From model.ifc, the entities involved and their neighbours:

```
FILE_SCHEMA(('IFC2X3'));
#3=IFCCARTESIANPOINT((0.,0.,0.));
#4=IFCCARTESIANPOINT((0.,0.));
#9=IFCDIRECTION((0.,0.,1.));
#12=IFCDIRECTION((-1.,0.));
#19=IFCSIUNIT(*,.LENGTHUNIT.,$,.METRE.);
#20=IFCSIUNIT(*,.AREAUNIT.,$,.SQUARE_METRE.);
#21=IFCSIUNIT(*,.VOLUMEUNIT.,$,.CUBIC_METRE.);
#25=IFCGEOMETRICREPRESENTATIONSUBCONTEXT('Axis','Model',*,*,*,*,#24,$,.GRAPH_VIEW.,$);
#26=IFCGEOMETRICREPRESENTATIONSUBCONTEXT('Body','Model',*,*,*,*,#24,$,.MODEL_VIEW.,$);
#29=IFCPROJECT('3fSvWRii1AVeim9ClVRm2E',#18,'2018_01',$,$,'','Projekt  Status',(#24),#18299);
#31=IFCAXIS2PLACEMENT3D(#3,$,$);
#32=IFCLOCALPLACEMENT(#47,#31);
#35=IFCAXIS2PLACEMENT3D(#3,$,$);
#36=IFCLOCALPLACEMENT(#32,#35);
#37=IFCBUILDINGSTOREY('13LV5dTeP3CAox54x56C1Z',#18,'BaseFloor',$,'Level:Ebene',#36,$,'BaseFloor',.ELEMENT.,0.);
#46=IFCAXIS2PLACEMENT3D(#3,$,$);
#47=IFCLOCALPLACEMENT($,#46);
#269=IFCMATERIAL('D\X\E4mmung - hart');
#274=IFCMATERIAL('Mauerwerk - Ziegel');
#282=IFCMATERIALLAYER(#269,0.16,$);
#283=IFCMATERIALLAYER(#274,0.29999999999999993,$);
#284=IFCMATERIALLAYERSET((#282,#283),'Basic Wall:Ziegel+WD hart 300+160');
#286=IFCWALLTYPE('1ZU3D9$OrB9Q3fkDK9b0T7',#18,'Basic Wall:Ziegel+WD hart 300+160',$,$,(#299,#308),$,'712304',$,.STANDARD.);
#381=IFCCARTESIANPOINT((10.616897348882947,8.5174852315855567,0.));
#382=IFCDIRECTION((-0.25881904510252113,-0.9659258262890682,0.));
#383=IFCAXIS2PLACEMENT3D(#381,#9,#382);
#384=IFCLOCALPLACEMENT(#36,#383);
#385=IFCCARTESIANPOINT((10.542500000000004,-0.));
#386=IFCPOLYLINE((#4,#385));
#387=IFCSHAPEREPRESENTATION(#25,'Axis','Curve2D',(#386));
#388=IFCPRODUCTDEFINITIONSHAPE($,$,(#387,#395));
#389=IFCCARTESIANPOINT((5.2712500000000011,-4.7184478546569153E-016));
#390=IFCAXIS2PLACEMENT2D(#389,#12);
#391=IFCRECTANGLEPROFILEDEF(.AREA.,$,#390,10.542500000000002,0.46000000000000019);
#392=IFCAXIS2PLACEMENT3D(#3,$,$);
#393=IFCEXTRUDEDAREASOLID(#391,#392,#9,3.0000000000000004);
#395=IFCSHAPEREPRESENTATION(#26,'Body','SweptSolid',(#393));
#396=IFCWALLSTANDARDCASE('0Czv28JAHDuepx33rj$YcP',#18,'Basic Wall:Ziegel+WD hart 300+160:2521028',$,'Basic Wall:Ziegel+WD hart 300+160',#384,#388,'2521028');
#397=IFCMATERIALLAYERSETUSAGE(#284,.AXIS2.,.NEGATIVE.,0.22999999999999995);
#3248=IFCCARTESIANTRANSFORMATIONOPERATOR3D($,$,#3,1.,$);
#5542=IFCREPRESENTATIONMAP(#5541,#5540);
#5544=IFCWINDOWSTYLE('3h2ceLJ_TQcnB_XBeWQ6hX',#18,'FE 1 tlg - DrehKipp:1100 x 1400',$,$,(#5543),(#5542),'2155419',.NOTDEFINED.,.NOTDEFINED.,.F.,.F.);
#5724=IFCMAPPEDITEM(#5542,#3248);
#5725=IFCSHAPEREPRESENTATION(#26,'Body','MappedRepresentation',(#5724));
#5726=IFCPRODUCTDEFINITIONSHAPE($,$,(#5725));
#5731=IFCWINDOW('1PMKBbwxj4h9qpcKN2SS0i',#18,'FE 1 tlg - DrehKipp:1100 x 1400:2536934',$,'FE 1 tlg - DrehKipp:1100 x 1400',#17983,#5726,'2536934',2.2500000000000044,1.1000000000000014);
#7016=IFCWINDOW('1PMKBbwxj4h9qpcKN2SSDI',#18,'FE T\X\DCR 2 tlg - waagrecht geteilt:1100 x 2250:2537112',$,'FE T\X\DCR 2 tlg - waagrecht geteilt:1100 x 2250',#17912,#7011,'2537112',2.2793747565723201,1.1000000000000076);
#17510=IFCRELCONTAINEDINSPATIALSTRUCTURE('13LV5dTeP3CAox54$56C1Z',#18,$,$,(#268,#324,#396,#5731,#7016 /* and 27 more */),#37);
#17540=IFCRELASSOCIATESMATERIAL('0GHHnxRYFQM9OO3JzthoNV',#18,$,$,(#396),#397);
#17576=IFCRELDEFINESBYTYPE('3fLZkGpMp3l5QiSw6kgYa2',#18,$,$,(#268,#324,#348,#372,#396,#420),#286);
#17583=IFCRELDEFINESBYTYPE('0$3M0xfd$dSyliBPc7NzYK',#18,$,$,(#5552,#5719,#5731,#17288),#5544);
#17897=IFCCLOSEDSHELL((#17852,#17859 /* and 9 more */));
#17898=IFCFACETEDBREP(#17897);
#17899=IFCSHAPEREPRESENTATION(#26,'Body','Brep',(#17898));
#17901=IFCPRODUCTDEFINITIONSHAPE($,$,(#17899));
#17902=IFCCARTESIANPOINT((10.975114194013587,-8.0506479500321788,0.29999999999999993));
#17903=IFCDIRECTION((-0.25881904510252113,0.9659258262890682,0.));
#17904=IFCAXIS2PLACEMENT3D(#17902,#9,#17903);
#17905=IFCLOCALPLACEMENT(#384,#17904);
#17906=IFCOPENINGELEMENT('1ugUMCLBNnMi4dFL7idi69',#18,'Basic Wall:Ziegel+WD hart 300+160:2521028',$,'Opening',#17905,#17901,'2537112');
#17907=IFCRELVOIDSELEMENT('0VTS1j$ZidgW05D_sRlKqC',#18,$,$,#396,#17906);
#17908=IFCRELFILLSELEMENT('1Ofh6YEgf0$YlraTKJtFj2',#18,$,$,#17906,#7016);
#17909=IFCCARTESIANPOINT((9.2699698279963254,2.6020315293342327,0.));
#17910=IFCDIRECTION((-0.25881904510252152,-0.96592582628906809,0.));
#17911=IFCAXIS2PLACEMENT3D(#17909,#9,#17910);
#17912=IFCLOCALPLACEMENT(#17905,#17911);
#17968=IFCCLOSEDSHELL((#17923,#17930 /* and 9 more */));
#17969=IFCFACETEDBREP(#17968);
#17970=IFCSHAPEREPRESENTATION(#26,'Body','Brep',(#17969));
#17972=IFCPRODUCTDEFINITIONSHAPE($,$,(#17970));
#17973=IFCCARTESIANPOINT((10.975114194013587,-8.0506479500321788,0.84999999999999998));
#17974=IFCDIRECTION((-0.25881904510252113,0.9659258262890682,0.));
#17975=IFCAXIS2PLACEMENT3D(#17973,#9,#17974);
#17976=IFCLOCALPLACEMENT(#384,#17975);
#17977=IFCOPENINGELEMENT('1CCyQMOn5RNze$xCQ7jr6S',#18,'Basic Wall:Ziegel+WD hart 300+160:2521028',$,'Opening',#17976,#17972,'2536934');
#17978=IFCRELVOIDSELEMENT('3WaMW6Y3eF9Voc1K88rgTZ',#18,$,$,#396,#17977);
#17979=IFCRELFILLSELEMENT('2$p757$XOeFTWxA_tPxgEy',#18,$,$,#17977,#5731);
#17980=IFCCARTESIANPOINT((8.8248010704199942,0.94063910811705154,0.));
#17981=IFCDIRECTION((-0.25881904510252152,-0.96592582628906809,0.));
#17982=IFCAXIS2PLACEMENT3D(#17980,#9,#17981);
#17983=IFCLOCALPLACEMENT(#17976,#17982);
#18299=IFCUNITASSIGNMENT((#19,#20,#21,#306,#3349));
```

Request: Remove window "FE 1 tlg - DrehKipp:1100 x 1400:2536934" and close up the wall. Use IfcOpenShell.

```python
import ifcopenshell
import ifcopenshell.api.feature
import ifcopenshell.api.root
import ifcopenshell.geom
import ifcopenshell.util.shape

model = ifcopenshell.open("model.ifc")
settings = ifcopenshell.geom.settings()


def volume(element):
    """Net volume in cubic metres, openings subtracted."""
    shape = ifcopenshell.geom.create_shape(settings, element)
    return ifcopenshell.util.shape.get_volume(shape.geometry)


window = model.by_id(5731)
opening = window.FillsVoids[0].RelatingOpeningElement
wall = opening.VoidsElements[0].RelatingBuildingElement
before = volume(wall)

ifcopenshell.api.root.remove_product(model, product=window)
ifcopenshell.api.feature.remove_feature(model, feature=opening)

after = volume(wall)

print(f"wall volume {before:.3f} -> {after:.3f} m3")

model.write("model-out.ifc")
```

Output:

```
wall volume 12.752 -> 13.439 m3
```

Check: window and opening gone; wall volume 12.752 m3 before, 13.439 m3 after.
